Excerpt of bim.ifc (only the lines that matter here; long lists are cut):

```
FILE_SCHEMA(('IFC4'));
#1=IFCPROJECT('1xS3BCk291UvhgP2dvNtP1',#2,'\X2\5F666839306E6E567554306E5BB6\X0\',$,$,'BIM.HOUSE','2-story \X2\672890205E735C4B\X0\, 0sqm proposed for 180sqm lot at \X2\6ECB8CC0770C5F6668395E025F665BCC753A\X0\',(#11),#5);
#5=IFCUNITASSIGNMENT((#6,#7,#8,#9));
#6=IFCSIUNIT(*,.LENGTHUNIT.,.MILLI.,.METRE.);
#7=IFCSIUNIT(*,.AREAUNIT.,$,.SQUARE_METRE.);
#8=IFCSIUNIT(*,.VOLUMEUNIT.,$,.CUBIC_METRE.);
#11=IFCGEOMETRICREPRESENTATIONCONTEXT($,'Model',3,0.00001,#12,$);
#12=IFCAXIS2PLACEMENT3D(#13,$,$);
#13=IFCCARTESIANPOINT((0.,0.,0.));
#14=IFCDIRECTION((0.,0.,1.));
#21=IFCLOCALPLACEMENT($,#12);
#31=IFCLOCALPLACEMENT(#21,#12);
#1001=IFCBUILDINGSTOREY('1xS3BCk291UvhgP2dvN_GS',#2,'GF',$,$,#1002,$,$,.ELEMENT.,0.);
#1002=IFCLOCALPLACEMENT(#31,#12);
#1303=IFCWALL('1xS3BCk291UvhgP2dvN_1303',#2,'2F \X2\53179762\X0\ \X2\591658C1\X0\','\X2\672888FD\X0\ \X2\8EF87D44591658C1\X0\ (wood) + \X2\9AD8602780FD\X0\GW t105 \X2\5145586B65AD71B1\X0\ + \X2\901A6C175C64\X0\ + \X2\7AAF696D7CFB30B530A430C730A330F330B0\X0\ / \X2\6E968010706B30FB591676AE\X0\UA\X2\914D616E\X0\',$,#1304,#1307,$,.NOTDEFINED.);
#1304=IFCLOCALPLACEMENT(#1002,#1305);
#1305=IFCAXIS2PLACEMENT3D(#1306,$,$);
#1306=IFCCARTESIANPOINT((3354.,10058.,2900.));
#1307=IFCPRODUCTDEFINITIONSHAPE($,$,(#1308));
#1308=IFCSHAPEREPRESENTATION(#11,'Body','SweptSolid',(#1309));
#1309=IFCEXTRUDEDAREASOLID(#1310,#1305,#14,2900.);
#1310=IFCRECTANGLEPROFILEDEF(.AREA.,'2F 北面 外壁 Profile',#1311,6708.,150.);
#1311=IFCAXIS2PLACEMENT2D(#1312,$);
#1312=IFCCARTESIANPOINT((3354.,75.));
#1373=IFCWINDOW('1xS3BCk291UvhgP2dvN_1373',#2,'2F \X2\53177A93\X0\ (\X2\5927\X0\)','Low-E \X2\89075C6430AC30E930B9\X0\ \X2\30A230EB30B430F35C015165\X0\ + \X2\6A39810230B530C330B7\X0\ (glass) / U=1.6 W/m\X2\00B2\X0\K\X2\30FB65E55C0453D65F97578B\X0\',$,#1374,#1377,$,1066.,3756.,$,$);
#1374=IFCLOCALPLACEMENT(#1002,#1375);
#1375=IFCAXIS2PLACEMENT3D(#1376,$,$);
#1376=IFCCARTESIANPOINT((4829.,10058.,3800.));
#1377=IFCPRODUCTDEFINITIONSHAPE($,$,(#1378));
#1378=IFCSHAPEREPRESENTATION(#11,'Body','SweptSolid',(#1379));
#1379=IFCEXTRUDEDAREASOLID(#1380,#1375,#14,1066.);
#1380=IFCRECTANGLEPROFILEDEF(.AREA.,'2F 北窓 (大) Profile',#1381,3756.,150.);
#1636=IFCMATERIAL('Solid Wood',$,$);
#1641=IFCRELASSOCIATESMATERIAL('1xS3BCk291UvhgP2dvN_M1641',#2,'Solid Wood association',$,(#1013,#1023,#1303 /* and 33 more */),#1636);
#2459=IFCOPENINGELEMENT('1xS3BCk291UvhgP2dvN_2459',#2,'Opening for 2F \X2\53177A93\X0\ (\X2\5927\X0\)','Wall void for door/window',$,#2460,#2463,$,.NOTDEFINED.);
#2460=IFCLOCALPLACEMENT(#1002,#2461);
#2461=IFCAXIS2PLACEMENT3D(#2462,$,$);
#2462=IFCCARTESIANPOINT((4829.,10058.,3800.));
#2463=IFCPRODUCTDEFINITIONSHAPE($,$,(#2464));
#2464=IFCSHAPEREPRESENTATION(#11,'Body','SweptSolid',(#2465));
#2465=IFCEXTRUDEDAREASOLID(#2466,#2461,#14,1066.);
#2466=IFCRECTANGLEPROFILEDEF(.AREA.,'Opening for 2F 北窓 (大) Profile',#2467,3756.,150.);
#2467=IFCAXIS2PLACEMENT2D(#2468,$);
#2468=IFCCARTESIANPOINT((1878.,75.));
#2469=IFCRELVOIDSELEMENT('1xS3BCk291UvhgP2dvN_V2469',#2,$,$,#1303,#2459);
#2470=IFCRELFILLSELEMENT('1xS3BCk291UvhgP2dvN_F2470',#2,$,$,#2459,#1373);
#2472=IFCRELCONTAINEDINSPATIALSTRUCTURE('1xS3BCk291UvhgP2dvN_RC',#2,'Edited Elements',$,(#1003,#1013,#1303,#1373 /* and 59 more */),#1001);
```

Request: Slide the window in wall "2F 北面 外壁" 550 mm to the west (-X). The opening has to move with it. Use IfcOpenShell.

```python
import ifcopenshell
import ifcopenshell.api.geometry
import ifcopenshell.util.placement
import ifcopenshell.util.unit

model = ifcopenshell.open("bim.ifc")
unit_scale = ifcopenshell.util.unit.calculate_unit_scale(model)

window = model.by_id(1373)
opening = window.FillsVoids[0].RelatingOpeningElement
wall = opening.VoidsElements[0].RelatingBuildingElement

wall_matrix = ifcopenshell.util.placement.get_local_placement(wall.ObjectPlacement)
shift = wall_matrix[:3, 0] * -0.55 / unit_scale
before = ifcopenshell.util.placement.get_local_placement(window.ObjectPlacement)[:3, 3].copy()

# The window is not placed relative to its opening, so move both.
for product in (opening, window):
    matrix = ifcopenshell.util.placement.get_local_placement(product.ObjectPlacement)
    matrix[:3, 3] += shift
    ifcopenshell.api.geometry.edit_object_placement(model, product=product, matrix=matrix, is_si=False)

after = ifcopenshell.util.placement.get_local_placement(window.ObjectPlacement)[:3, 3]
print("window moved by", (after - before).round(3) + 0.0)

model.write("bim-out.ifc")
```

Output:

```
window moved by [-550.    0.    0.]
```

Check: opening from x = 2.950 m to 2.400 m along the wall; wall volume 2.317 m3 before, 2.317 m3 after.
